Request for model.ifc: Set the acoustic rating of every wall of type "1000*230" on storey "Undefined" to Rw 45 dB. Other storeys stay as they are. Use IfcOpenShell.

First a look at what the model holds.

```python
import ifcopenshell
import ifcopenshell.util.element

model = ifcopenshell.open("model.ifc")
print(model.schema)
storey = next(s for s in model.by_type("IfcBuildingStorey") if s.Name == "Undefined")
walls = [e for e in ifcopenshell.util.element.get_decomposition(storey) if e.is_a("IfcWall")]
seen = {}
for e in walls:
    element_type = ifcopenshell.util.element.get_type(e)
    key = (element_type.Name if element_type != e and element_type else None, ifcopenshell.util.element.get_pset(e, "Pset_WallCommon", "AcousticRating"))
    seen[key] = seen.get(key, 0) + 1
for (name, value), count in sorted(seen.items(), key=str):
    print(count, "x", name, "|", value)
```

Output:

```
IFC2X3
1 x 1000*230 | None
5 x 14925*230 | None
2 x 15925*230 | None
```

```python
import ifcopenshell
import ifcopenshell.api.pset
import ifcopenshell.util.element

model = ifcopenshell.open("model.ifc")

storey = next(s for s in model.by_type("IfcBuildingStorey") if s.Name == "Undefined")
walls = [e for e in ifcopenshell.util.element.get_decomposition(storey) if e.is_a("IfcWall")]

count = 0
for e in walls:
    element_type = ifcopenshell.util.element.get_type(e)
    if element_type in (None, e) or element_type.Name != "1000*230":
        continue
    # add_pset returns the element's existing set when there is one.
    pset = ifcopenshell.api.pset.add_pset(model, product=e, name="Pset_WallCommon")
    ifcopenshell.api.pset.edit_pset(model, pset=pset, properties={"AcousticRating": "Rw 45 dB"})
    count += 1

print(count, "walls updated")

model.write("model_v2.ifc")
```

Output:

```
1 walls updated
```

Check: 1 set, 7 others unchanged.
